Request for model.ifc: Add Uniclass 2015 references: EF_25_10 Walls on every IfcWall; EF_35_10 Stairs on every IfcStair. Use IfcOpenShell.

First a look at what the model holds.

```python
import ifcopenshell

model = ifcopenshell.open("model.ifc")
print(model.schema)
print("classifications:", [c.Name for c in model.by_type("IfcClassification")])
for ifc_class in ("IfcDoor", "IfcRoof", "IfcStair", "IfcWall", "IfcWindow"):
    print(ifc_class, len(model.by_type(ifc_class)))
```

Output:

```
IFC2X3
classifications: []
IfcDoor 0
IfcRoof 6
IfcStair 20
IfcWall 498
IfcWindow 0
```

```python
import ifcopenshell
import ifcopenshell.api.classification

model = ifcopenshell.open("model.ifc")

# IFC2X3 requires Source and Edition and has no link from the project to the system.
system = model.create_entity("IfcClassification", Source="NBS", Edition="2015", Name="Uniclass 2015")

codes = {
    "IfcWall": ("EF_25_10", "Walls"),
    "IfcStair": ("EF_35_10", "Stairs"),
}
for ifc_class, (code, name) in codes.items():
    products = model.by_type(ifc_class)
    ifcopenshell.api.classification.add_reference(
        model, products=products, classification=system, identification=code, name=name
    )
    print(code, len(products))

model.write("model_updated.ifc")
```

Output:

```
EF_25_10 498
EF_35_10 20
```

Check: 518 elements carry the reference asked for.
